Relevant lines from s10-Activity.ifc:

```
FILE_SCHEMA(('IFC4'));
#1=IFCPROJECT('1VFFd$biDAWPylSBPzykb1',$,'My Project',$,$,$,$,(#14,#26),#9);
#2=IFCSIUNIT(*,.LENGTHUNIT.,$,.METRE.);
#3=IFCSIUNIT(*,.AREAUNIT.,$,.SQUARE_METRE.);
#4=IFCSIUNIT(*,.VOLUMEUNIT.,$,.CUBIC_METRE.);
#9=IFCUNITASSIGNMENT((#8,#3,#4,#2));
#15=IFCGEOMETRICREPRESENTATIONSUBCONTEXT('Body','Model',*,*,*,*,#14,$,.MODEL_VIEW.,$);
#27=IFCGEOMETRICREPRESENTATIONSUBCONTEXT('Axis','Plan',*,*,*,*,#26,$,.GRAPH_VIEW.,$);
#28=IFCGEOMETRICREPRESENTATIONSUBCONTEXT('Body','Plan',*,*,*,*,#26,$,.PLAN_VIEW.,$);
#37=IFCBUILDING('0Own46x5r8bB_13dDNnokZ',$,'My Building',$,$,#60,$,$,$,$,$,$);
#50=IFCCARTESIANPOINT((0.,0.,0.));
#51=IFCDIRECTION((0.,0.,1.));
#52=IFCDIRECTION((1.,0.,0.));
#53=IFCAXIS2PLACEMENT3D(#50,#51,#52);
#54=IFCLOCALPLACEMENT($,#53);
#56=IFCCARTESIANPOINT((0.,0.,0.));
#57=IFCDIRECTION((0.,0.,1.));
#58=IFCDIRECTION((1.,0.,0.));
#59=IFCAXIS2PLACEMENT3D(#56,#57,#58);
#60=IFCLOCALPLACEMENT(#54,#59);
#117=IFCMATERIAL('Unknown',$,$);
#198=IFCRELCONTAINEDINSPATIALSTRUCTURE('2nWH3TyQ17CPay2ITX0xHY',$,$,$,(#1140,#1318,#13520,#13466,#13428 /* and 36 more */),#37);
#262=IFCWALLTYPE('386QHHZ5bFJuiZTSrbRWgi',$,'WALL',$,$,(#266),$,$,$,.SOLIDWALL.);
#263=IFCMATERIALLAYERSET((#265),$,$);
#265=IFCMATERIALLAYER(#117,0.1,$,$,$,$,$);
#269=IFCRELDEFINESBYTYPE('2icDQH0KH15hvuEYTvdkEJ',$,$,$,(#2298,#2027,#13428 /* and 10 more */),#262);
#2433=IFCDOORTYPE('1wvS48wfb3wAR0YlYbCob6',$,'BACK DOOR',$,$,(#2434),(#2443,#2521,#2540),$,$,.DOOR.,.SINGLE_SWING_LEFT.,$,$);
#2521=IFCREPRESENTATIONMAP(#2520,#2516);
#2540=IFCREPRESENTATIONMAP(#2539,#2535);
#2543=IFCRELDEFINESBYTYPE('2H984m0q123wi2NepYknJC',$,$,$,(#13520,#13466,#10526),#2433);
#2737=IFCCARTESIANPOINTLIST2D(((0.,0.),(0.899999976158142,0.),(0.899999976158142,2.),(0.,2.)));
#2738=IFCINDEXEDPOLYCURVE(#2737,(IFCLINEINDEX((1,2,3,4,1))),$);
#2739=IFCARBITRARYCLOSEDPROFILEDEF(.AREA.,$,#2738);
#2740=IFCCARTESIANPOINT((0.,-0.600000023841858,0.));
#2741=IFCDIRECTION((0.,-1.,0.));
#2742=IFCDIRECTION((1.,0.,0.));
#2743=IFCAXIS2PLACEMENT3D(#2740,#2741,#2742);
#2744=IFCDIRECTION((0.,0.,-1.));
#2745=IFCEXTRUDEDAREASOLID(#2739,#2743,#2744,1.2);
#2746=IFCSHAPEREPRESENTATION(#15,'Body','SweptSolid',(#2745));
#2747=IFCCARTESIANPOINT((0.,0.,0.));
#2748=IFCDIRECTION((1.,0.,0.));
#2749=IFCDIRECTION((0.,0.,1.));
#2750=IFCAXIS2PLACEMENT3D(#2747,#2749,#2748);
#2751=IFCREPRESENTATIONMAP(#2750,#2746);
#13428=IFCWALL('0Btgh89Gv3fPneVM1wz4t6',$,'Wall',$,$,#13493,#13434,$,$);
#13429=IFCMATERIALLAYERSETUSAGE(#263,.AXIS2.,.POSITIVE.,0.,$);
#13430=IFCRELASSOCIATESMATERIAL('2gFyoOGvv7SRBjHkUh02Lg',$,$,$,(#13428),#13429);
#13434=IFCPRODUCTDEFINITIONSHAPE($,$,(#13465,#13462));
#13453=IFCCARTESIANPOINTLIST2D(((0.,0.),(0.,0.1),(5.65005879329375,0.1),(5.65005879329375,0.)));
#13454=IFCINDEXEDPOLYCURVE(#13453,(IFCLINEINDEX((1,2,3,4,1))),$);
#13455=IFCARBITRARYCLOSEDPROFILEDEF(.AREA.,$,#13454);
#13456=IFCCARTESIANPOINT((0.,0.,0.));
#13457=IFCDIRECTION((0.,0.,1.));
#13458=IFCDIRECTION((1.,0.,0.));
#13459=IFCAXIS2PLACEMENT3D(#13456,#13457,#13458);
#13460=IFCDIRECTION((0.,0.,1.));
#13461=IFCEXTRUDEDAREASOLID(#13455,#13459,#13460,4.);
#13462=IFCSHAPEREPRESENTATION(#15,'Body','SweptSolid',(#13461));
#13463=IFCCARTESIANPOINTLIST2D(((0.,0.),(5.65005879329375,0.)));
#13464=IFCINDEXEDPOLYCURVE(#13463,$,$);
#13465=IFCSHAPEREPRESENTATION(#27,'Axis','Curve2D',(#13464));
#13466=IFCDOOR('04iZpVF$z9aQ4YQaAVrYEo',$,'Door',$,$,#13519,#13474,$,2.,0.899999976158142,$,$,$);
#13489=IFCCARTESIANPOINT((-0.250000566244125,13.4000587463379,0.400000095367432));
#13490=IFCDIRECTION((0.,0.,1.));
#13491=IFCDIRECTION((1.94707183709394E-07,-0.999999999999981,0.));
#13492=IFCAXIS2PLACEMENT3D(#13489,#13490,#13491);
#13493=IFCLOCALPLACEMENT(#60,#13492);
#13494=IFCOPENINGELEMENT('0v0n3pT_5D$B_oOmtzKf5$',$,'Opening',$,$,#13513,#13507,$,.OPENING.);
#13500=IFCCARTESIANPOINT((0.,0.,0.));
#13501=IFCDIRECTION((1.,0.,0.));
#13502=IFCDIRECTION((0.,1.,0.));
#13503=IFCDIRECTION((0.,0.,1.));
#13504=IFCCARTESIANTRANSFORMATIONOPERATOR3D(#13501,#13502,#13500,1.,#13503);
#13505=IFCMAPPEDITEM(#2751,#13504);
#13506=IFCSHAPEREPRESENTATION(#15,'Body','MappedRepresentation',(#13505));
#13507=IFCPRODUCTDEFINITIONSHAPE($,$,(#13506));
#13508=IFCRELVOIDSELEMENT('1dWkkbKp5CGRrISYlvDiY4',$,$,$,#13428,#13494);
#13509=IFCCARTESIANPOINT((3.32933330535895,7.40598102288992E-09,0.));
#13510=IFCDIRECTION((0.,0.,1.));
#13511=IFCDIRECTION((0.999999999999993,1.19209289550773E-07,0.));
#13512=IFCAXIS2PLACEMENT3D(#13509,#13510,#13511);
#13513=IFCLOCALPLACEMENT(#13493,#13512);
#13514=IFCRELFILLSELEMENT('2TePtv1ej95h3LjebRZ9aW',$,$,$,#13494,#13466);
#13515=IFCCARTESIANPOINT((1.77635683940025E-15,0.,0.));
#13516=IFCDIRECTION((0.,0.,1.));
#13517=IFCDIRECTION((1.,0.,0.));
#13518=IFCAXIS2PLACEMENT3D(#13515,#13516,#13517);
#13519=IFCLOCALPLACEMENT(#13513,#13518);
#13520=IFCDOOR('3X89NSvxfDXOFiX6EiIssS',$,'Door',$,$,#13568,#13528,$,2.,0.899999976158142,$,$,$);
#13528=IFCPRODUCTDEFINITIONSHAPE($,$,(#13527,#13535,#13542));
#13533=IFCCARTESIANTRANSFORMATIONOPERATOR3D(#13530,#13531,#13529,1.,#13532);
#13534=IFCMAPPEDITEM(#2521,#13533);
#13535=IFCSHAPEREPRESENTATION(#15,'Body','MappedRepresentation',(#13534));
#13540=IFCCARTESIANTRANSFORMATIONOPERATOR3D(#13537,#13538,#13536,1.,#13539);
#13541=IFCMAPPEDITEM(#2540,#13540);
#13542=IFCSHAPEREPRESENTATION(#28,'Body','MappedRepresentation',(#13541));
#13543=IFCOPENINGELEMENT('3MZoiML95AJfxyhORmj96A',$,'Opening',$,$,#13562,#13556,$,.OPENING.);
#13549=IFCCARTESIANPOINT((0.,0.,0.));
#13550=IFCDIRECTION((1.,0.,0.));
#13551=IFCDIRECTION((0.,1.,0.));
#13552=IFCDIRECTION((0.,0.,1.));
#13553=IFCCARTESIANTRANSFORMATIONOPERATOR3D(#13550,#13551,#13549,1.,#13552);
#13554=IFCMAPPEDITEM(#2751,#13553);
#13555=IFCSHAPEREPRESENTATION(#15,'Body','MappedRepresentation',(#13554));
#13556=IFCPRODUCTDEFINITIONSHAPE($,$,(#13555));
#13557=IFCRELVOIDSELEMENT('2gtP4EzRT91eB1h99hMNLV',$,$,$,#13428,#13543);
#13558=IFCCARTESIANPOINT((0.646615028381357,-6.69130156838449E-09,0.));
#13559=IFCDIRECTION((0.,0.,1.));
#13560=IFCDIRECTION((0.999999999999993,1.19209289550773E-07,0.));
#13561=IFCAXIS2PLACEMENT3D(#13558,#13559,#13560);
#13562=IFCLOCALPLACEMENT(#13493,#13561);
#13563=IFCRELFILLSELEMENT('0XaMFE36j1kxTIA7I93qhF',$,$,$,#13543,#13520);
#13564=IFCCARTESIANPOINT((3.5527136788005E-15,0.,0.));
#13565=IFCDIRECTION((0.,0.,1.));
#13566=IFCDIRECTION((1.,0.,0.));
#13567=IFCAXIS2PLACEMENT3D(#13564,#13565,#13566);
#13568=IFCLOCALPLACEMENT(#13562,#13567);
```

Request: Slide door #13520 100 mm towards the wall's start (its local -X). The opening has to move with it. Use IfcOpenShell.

```python
import ifcopenshell
import ifcopenshell.api.geometry
import ifcopenshell.util.placement
import ifcopenshell.util.unit

model = ifcopenshell.open("s10-Activity.ifc")
unit_scale = ifcopenshell.util.unit.calculate_unit_scale(model)

door = model.by_guid("3X89NSvxfDXOFiX6EiIssS")
opening = door.FillsVoids[0].RelatingOpeningElement
wall = opening.VoidsElements[0].RelatingBuildingElement

wall_matrix = ifcopenshell.util.placement.get_local_placement(wall.ObjectPlacement)
shift = wall_matrix[:3, 0] * -0.1 / unit_scale
before = ifcopenshell.util.placement.get_local_placement(door.ObjectPlacement)[:3, 3].copy()

# The door is placed relative to its opening, so it follows when the opening moves.
matrix = ifcopenshell.util.placement.get_local_placement(opening.ObjectPlacement)
matrix[:3, 3] += shift
ifcopenshell.api.geometry.edit_object_placement(
    model, product=opening, matrix=matrix, is_si=False, should_transform_children=True
)

after = ifcopenshell.util.placement.get_local_placement(door.ObjectPlacement)[:3, 3]
print("door moved by", (after - before).round(3) + 0.0)

model.write("s10-Activity_updated.ifc")
```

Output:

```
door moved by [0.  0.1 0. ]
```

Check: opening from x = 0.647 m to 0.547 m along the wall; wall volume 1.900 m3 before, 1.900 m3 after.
